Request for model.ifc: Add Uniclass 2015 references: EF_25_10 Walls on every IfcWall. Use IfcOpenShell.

First a look at what the model holds.

```python
import ifcopenshell

model = ifcopenshell.open("model.ifc")
print(model.schema)
print("classifications:", [c.Name for c in model.by_type("IfcClassification")])
for ifc_class in ("IfcDoor", "IfcRoof", "IfcStair", "IfcWall", "IfcWindow"):
    print(ifc_class, len(model.by_type(ifc_class)))
```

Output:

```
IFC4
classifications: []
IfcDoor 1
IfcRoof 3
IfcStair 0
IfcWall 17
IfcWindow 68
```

```python
import ifcopenshell
import ifcopenshell.api.classification

model = ifcopenshell.open("model.ifc")

system = ifcopenshell.api.classification.add_classification(model, classification="Uniclass 2015")

codes = {
    "IfcWall": ("EF_25_10", "Walls"),
}
for ifc_class, (code, name) in codes.items():
    products = model.by_type(ifc_class)
    ifcopenshell.api.classification.add_reference(
        model, products=products, classification=system, identification=code, name=name
    )
    print(code, len(products))

model.write("model-out.ifc")
```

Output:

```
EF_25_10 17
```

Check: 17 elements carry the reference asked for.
